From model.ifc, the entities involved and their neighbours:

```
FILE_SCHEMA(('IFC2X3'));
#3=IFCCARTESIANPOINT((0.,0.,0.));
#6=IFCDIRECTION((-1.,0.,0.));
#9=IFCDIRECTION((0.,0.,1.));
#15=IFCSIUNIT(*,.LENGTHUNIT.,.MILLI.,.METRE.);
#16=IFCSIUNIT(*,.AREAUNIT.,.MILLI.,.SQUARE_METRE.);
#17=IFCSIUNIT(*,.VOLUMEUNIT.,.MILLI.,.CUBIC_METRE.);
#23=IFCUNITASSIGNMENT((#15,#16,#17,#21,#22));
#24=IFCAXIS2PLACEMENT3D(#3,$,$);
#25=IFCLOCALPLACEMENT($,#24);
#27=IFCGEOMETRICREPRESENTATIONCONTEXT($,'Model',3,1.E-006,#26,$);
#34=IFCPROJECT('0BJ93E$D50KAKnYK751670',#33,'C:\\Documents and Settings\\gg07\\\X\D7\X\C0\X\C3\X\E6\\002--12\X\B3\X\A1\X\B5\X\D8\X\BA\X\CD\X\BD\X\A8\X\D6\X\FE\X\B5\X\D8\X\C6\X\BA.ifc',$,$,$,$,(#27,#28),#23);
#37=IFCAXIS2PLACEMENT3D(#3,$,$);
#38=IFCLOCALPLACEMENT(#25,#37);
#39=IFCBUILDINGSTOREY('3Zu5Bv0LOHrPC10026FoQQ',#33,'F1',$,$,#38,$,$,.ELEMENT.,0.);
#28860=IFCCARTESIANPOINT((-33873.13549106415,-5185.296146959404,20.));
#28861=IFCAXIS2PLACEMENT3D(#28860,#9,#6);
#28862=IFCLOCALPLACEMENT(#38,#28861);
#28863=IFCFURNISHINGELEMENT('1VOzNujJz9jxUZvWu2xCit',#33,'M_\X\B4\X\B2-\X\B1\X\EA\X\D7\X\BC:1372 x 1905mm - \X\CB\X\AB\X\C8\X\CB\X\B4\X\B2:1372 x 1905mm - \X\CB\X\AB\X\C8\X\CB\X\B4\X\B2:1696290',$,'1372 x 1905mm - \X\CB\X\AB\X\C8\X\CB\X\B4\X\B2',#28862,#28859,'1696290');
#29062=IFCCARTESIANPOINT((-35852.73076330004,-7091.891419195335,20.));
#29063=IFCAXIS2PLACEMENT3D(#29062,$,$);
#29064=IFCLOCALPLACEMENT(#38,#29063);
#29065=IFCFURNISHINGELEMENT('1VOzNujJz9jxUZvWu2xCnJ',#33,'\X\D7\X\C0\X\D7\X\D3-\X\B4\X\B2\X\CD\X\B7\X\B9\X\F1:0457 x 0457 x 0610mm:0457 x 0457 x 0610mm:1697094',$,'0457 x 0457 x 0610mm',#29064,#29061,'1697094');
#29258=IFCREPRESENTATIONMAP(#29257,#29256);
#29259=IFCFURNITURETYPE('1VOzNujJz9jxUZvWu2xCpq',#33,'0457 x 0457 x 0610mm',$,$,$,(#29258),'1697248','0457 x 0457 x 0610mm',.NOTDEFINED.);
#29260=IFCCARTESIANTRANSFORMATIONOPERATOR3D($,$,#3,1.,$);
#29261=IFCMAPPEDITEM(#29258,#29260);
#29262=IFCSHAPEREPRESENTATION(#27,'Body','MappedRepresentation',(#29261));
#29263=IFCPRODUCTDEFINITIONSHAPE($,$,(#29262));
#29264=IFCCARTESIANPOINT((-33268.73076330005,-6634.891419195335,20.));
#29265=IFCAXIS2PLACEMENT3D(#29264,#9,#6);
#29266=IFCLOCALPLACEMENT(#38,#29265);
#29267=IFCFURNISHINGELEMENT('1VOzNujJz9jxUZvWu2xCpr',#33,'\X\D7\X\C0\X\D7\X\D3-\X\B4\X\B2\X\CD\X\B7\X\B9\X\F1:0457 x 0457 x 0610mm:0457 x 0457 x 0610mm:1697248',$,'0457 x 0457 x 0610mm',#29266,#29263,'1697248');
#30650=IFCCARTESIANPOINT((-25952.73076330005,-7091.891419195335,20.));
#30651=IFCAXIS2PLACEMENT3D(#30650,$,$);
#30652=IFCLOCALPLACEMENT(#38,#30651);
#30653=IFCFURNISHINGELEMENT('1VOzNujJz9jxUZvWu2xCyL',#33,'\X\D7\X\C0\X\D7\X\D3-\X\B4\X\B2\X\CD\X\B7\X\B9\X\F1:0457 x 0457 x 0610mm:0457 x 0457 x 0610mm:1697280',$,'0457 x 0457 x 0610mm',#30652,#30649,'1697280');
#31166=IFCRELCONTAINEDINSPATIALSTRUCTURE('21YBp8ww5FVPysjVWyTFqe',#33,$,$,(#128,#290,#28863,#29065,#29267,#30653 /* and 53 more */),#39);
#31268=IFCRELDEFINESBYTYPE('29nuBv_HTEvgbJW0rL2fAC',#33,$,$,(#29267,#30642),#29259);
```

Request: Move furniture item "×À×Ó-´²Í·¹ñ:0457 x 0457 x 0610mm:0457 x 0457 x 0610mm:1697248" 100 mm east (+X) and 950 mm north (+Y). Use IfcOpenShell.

```python
import ifcopenshell
import ifcopenshell.api.geometry
import ifcopenshell.util.placement

model = ifcopenshell.open("model.ifc")

item = model.by_guid("1VOzNujJz9jxUZvWu2xCpr")
matrix = ifcopenshell.util.placement.get_local_placement(item.ObjectPlacement)
matrix[0, 3] += 100.0
matrix[1, 3] += 950.0
ifcopenshell.api.geometry.edit_object_placement(model, product=item, matrix=matrix, is_si=False)

print(ifcopenshell.util.placement.get_local_placement(item.ObjectPlacement).round(3) + 0.0)

model.write("model_v2.ifc")
```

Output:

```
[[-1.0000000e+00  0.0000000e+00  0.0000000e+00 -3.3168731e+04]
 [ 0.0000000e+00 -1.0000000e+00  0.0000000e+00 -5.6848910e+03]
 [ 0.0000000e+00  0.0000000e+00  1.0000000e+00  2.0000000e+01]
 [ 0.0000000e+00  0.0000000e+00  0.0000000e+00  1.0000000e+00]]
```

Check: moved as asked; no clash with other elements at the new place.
